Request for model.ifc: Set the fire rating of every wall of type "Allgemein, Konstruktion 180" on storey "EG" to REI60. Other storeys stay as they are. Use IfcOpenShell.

First a look at what the model holds.

```python
import ifcopenshell
import ifcopenshell.util.element

model = ifcopenshell.open("model.ifc")
print(model.schema)
storey = next(s for s in model.by_type("IfcBuildingStorey") if s.Name == "EG")
walls = [e for e in ifcopenshell.util.element.get_decomposition(storey) if e.is_a("IfcWall")]
seen = {}
for e in walls:
    element_type = ifcopenshell.util.element.get_type(e)
    key = (element_type.Name if element_type != e and element_type else None, ifcopenshell.util.element.get_pset(e, "Pset_WallCommon", "FireRating"))
    seen[key] = seen.get(key, 0) + 1
for (name, value), count in sorted(seen.items(), key=str):
    print(count, "x", name, "|", value)
```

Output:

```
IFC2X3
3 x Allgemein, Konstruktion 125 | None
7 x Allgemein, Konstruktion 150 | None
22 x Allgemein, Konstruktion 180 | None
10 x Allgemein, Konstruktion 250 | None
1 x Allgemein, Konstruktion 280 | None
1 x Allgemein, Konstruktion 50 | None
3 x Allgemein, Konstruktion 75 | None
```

```python
import ifcopenshell
import ifcopenshell.api.pset
import ifcopenshell.util.element

model = ifcopenshell.open("model.ifc")

storey = next(s for s in model.by_type("IfcBuildingStorey") if s.Name == "EG")
walls = [e for e in ifcopenshell.util.element.get_decomposition(storey) if e.is_a("IfcWall")]

count = 0
for e in walls:
    element_type = ifcopenshell.util.element.get_type(e)
    if element_type in (None, e) or element_type.Name != "Allgemein, Konstruktion 180":
        continue
    # add_pset returns the element's existing set when there is one.
    pset = ifcopenshell.api.pset.add_pset(model, product=e, name="Pset_WallCommon")
    ifcopenshell.api.pset.edit_pset(model, pset=pset, properties={"FireRating": "REI60"})
    count += 1

print(count, "walls updated")

model.write("model-out.ifc")
```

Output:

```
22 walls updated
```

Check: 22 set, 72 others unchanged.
